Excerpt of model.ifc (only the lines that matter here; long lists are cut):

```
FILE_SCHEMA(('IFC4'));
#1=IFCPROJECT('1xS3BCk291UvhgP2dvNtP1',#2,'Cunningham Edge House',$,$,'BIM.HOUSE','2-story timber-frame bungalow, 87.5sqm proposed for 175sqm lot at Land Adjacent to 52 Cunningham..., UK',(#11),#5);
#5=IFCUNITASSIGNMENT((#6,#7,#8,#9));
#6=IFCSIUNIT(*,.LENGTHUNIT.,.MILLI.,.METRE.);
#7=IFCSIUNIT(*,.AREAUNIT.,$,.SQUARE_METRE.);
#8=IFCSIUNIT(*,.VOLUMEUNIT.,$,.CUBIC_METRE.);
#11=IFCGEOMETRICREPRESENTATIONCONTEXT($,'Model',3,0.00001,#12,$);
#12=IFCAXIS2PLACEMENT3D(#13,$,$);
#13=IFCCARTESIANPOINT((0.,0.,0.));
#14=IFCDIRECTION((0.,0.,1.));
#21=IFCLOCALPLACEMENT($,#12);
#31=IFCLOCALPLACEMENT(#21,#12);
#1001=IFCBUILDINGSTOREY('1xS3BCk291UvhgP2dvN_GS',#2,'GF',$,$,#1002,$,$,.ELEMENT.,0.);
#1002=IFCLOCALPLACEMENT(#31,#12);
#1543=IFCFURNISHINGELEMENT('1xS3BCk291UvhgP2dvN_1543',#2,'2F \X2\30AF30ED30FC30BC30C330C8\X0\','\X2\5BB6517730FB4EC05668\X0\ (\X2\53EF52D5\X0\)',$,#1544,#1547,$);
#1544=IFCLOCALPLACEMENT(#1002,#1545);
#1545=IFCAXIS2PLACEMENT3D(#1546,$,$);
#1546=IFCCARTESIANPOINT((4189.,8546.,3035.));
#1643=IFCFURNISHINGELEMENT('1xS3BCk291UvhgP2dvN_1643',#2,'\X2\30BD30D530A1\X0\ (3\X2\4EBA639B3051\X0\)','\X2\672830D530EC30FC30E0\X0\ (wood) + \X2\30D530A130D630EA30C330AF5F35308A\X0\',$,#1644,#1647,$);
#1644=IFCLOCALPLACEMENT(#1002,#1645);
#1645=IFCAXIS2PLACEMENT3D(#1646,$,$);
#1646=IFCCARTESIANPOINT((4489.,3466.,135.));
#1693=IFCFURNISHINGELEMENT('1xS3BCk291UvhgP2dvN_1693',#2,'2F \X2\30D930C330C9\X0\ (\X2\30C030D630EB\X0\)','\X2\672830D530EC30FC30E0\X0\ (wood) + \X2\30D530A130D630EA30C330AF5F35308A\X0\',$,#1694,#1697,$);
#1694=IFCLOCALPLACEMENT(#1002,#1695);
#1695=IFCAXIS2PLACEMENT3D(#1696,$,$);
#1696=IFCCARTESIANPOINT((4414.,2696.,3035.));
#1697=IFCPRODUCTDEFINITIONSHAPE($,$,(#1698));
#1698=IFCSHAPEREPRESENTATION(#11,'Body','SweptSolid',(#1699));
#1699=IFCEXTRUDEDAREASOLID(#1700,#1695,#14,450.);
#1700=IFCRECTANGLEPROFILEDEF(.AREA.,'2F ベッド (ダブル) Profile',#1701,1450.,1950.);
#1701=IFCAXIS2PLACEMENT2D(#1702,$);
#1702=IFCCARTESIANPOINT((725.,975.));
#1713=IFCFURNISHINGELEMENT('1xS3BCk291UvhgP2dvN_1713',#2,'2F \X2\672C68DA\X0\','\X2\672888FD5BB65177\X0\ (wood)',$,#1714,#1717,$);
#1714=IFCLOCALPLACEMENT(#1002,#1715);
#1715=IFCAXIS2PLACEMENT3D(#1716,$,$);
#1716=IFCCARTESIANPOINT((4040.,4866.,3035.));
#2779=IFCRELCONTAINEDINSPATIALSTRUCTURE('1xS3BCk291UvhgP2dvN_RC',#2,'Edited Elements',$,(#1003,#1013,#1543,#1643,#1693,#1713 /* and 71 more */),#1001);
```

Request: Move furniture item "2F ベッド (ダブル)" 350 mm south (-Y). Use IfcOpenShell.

```python
import ifcopenshell
import ifcopenshell.api.geometry
import ifcopenshell.util.placement
import ifcopenshell.util.unit

model = ifcopenshell.open("model.ifc")
unit_scale = ifcopenshell.util.unit.calculate_unit_scale(model)

item = model.by_id(1693)
matrix = ifcopenshell.util.placement.get_local_placement(item.ObjectPlacement)
matrix[1, 3] -= 0.35 / unit_scale
ifcopenshell.api.geometry.edit_object_placement(model, product=item, matrix=matrix, is_si=False)

print(ifcopenshell.util.placement.get_local_placement(item.ObjectPlacement).round(3) + 0.0)

model.write("model_v2.ifc")
```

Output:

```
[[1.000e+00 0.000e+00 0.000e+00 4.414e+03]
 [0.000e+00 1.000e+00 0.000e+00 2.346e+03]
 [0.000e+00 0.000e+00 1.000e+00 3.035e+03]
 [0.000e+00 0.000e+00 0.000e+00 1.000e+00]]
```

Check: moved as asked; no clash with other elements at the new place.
